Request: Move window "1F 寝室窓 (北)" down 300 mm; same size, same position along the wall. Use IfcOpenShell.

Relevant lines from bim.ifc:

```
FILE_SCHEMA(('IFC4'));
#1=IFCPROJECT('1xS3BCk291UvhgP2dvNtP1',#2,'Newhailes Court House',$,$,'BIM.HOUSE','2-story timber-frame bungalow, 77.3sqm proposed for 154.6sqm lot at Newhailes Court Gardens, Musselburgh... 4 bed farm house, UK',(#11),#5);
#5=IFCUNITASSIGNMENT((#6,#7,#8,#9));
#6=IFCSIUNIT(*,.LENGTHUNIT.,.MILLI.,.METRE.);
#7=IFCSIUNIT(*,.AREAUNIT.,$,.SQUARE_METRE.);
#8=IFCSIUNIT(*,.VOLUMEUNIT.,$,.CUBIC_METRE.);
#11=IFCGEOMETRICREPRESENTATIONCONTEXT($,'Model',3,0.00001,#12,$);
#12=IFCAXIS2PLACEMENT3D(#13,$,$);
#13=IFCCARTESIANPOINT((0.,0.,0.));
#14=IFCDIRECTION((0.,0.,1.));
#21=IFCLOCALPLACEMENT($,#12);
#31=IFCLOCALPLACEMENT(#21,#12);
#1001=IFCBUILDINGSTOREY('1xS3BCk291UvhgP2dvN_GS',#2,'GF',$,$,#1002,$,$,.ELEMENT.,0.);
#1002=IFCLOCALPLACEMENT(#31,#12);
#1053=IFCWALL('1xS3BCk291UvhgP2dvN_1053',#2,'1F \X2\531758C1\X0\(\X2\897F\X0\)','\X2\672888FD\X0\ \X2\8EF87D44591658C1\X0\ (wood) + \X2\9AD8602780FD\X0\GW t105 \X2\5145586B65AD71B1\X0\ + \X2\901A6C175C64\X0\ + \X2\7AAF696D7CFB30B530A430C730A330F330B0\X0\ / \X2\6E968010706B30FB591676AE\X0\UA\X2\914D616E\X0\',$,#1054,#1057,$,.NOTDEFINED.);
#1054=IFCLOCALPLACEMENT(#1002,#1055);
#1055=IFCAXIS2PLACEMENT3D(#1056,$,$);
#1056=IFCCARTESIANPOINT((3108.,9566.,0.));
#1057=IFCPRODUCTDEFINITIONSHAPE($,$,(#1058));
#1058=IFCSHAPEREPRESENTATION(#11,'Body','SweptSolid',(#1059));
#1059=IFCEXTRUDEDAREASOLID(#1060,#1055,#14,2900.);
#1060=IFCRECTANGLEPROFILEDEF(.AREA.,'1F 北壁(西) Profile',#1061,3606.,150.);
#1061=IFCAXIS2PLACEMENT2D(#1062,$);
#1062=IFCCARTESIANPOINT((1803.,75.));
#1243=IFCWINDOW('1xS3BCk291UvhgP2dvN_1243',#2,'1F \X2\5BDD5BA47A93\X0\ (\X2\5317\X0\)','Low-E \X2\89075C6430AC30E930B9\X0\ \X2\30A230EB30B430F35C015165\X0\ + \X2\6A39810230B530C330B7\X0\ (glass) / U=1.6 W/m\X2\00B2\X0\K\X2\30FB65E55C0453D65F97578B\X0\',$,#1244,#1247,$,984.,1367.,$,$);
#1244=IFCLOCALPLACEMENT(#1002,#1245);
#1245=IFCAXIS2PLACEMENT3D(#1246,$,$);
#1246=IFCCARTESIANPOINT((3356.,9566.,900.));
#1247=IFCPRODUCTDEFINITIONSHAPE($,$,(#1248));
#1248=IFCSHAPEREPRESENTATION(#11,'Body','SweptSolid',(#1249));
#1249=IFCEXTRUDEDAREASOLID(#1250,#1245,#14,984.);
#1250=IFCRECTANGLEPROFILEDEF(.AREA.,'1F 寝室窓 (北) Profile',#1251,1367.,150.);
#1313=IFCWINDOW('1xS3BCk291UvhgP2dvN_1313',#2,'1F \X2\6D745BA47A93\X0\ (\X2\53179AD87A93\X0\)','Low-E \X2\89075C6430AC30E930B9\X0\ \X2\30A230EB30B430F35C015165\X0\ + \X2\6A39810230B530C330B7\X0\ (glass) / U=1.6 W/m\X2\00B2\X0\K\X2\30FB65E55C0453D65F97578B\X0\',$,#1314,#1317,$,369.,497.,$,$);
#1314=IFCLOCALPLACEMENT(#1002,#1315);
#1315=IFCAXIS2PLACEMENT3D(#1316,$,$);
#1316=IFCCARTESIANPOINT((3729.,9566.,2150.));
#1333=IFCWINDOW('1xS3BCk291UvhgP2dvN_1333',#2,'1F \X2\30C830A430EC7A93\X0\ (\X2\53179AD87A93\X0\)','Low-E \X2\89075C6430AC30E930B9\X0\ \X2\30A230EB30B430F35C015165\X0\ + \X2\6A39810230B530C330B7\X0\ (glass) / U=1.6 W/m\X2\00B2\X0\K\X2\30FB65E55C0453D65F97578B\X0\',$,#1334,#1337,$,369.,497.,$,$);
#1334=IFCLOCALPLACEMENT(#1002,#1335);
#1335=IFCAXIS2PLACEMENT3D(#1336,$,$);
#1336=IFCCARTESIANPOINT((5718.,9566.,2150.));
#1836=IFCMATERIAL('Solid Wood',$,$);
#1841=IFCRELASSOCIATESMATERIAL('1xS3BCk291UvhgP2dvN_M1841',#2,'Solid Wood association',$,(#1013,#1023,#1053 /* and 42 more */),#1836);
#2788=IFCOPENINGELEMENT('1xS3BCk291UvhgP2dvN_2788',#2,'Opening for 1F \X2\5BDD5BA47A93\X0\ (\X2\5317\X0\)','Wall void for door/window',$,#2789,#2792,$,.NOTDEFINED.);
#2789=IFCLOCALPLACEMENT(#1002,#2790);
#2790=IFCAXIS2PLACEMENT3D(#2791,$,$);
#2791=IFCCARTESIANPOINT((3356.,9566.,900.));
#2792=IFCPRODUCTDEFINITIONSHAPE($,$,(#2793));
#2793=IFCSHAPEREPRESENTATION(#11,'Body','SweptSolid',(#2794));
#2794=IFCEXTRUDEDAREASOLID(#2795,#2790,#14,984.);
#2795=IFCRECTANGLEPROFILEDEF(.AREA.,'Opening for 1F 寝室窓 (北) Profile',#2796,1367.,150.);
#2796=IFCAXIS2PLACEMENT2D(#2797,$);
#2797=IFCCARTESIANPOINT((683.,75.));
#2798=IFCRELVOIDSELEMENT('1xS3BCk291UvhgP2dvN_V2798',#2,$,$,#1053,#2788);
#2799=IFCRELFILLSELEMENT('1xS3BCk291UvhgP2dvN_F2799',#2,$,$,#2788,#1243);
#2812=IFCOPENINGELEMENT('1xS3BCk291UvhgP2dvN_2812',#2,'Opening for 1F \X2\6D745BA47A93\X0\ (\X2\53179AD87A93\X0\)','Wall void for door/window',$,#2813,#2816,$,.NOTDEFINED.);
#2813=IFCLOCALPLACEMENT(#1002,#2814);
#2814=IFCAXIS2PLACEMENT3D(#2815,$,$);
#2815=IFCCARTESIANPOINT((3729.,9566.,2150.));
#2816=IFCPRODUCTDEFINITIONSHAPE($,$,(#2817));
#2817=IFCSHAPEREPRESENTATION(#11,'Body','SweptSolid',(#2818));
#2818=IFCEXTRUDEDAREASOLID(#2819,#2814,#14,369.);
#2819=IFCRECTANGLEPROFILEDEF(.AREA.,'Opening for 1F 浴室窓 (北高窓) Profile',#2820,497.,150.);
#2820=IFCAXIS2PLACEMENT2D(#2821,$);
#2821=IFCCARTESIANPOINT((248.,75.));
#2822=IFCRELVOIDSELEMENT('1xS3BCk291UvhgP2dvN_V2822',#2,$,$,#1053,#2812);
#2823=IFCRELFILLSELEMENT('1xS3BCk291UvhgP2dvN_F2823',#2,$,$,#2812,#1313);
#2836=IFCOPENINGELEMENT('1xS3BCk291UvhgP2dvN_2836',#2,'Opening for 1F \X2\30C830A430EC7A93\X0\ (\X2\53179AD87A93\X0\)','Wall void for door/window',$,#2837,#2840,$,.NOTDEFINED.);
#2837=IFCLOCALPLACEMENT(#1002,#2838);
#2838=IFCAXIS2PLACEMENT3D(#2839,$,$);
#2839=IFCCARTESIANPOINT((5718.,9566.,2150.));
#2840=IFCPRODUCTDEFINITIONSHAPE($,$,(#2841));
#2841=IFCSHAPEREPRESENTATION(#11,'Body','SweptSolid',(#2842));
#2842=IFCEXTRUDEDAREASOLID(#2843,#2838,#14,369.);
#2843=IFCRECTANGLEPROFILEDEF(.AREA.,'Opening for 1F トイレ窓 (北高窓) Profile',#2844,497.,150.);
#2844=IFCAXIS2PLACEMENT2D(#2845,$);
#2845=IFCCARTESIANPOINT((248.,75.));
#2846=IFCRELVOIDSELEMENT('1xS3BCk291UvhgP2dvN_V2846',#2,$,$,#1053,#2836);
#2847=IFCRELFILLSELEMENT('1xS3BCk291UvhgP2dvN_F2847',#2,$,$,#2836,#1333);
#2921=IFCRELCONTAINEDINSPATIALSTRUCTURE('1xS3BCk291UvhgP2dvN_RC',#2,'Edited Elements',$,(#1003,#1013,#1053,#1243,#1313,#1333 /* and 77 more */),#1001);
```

```python
import numpy as np
import ifcopenshell
import ifcopenshell.api.geometry
import ifcopenshell.util.placement
import ifcopenshell.util.unit

model = ifcopenshell.open("bim.ifc")
unit_scale = ifcopenshell.util.unit.calculate_unit_scale(model)

window = model.by_guid("1xS3BCk291UvhgP2dvN_1243")
opening = window.FillsVoids[0].RelatingOpeningElement
dz = -0.3 / unit_scale

shift = np.array([0.0, 0.0, dz])
# The window is not placed relative to its opening, so move both.
for product in (opening, window):
    matrix = ifcopenshell.util.placement.get_local_placement(product.ObjectPlacement)
    matrix[:3, 3] += shift
    ifcopenshell.api.geometry.edit_object_placement(model, product=product, matrix=matrix, is_si=False)

print(f"moved by {dz * unit_scale:+.3f} m")

model.write("bim-out.ifc")
```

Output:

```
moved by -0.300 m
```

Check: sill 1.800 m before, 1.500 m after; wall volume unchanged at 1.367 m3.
